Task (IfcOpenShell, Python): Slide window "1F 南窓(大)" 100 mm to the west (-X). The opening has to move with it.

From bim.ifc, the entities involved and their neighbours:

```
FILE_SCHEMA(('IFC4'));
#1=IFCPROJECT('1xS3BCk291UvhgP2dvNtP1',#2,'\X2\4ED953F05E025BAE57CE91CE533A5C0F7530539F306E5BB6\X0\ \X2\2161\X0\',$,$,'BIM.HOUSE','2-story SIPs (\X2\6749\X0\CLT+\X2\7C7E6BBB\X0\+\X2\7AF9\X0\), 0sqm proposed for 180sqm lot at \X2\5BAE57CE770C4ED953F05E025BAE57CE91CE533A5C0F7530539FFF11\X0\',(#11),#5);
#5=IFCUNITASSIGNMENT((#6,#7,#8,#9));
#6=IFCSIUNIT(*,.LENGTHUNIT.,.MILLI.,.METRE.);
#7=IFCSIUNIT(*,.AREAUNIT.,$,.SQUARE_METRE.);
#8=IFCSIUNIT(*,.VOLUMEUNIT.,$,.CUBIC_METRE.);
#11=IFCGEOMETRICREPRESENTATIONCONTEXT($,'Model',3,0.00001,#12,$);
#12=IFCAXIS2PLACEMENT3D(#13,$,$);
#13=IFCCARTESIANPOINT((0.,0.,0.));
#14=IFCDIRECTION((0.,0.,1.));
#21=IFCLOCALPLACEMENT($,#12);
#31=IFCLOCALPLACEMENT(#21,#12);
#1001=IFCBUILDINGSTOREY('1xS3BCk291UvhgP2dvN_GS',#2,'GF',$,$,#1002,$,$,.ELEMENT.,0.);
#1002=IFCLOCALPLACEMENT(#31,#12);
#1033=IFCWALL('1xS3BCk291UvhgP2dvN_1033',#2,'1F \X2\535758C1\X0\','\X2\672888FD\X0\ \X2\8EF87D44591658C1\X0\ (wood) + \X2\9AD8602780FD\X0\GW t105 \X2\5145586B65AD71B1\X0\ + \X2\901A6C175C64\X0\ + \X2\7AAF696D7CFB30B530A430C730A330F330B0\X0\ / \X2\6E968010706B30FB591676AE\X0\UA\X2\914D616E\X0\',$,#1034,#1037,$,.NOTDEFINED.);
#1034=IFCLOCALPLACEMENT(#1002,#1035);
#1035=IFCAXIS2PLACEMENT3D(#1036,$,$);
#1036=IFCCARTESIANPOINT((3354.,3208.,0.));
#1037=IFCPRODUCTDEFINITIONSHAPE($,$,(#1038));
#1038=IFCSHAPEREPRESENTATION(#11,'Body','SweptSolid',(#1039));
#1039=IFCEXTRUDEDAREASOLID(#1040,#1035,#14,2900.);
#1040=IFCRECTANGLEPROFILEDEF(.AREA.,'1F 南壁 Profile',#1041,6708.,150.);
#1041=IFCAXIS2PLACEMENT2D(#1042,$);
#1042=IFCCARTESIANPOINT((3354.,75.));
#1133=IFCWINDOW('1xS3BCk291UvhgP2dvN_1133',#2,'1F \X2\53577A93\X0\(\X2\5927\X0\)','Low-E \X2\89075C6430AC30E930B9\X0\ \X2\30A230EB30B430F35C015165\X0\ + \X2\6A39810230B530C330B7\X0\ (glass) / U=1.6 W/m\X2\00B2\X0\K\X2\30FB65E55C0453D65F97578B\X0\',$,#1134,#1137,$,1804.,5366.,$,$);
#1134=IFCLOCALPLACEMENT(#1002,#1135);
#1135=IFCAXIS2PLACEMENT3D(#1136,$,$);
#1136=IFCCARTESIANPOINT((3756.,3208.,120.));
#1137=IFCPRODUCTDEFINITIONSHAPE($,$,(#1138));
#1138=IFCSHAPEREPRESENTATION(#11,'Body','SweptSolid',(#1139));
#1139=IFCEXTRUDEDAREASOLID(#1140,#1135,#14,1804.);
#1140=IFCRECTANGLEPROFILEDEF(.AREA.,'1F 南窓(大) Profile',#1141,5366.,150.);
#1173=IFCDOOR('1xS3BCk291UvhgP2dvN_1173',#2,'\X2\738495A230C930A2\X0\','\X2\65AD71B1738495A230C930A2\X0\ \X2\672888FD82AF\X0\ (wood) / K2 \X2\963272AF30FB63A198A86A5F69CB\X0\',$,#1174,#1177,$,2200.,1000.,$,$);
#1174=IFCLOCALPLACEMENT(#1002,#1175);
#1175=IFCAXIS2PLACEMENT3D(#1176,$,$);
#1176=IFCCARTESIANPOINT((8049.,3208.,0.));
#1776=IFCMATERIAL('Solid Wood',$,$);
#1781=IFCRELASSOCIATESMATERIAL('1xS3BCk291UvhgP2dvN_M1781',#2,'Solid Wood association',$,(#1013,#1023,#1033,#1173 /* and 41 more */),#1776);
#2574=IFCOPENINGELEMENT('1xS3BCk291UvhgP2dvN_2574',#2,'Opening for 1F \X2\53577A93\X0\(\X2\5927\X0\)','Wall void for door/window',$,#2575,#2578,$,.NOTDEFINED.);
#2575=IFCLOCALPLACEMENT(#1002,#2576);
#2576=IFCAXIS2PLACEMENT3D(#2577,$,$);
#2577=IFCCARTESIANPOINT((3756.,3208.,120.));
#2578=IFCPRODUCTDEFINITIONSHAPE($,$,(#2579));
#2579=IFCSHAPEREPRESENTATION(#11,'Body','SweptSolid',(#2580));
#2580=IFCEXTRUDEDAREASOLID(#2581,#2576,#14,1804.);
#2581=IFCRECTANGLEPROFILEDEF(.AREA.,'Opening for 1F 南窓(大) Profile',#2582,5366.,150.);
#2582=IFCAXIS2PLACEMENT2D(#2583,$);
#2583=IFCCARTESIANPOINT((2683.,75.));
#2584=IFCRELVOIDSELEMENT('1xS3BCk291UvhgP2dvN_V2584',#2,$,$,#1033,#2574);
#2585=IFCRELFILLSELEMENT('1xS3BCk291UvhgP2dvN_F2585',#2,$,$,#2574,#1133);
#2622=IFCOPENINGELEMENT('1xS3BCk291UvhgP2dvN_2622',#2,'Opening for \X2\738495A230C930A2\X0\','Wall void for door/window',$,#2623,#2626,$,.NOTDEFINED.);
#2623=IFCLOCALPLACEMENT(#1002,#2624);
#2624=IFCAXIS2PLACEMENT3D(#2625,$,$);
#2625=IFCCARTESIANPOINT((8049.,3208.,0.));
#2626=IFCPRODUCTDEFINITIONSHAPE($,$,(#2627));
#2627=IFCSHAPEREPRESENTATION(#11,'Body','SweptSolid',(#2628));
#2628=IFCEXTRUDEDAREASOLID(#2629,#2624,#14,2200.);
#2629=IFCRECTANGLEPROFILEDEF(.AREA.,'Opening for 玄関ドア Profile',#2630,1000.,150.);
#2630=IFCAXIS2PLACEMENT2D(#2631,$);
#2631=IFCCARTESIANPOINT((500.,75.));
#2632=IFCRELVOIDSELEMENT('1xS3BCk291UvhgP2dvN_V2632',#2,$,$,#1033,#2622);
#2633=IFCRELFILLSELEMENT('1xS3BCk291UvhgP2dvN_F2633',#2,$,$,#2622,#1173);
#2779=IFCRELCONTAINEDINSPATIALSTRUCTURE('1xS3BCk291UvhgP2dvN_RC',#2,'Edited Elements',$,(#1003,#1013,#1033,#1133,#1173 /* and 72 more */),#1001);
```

```python
import ifcopenshell
import ifcopenshell.api.geometry
import ifcopenshell.util.placement
import ifcopenshell.util.unit

model = ifcopenshell.open("bim.ifc")
unit_scale = ifcopenshell.util.unit.calculate_unit_scale(model)

window = model.by_id(1133)
opening = window.FillsVoids[0].RelatingOpeningElement
wall = opening.VoidsElements[0].RelatingBuildingElement

wall_matrix = ifcopenshell.util.placement.get_local_placement(wall.ObjectPlacement)
shift = wall_matrix[:3, 0] * -0.1 / unit_scale
before = ifcopenshell.util.placement.get_local_placement(window.ObjectPlacement)[:3, 3].copy()

# The window is not placed relative to its opening, so move both.
for product in (opening, window):
    matrix = ifcopenshell.util.placement.get_local_placement(product.ObjectPlacement)
    matrix[:3, 3] += shift
    ifcopenshell.api.geometry.edit_object_placement(model, product=product, matrix=matrix, is_si=False)

after = ifcopenshell.util.placement.get_local_placement(window.ObjectPlacement)[:3, 3]
print("window moved by", (after - before).round(3) + 0.0)

model.write("bim_edited.ifc")
```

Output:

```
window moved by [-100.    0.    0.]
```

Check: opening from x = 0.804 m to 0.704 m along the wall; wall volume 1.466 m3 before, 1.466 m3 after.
